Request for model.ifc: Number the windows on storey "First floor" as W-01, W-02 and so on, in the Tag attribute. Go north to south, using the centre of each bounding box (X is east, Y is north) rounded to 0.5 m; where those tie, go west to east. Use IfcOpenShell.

First a look at what the model holds.

```python
import ifcopenshell
import ifcopenshell.util.element
import ifcopenshell.util.placement

model = ifcopenshell.open("model.ifc")
print(model.schema)
storey = next(s for s in model.by_type("IfcBuildingStorey") if s.Name == "First floor")
windows = [e for e in ifcopenshell.util.element.get_decomposition(storey) if e.is_a("IfcWindow")]
for e in sorted(windows, key=lambda e: e.id()):
    origin = ifcopenshell.util.placement.get_local_placement(e.ObjectPlacement)[:3, 3]
    print(e.id(), e.Tag, e.Name, origin.round(2) + 0.0, sep=" | ")
```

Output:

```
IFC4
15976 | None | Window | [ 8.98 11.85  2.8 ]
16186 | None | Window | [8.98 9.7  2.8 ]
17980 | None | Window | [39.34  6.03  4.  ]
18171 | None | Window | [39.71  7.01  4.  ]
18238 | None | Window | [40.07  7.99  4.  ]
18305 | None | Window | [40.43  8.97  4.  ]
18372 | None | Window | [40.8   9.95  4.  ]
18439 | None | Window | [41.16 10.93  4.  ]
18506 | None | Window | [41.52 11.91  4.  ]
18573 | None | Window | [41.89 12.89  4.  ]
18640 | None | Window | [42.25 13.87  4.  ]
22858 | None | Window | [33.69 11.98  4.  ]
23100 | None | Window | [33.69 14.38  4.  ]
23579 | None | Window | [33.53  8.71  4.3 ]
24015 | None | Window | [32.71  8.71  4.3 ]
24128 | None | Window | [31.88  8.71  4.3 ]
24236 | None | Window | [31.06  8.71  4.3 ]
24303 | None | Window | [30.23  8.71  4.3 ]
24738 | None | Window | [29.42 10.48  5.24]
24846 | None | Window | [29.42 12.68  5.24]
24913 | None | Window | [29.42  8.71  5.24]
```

```python
import ifcopenshell
import ifcopenshell.geom
import ifcopenshell.util.element
import ifcopenshell.util.shape

model = ifcopenshell.open("model.ifc")
settings = ifcopenshell.geom.settings()
settings.set("use-world-coords", True)


def centre(element):
    shape = ifcopenshell.geom.create_shape(settings, element)
    return ifcopenshell.util.shape.get_bbox_centroid(shape.geometry)


storey = next(s for s in model.by_type("IfcBuildingStorey") if s.Name == "First floor")
windows = [e for e in ifcopenshell.util.element.get_decomposition(storey) if e.is_a("IfcWindow")]

# Insertion points can sit at a corner or the storey origin, so sort by the geometry (in metres).
centres = {e: centre(e) for e in windows}
windows.sort(key=lambda e: (-round(centres[e][1] / 0.5), centres[e][0]))

for i, e in enumerate(windows, start=1):
    number = f"W-{i:02d}"
    e.Tag = number
    print(e.id(), number)

model.write("model_updated.ifc")
```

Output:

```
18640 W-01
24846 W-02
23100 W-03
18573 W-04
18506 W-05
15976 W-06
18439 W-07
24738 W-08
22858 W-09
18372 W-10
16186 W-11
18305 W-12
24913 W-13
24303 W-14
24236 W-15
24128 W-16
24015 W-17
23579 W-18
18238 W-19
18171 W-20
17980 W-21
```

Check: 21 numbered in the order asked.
